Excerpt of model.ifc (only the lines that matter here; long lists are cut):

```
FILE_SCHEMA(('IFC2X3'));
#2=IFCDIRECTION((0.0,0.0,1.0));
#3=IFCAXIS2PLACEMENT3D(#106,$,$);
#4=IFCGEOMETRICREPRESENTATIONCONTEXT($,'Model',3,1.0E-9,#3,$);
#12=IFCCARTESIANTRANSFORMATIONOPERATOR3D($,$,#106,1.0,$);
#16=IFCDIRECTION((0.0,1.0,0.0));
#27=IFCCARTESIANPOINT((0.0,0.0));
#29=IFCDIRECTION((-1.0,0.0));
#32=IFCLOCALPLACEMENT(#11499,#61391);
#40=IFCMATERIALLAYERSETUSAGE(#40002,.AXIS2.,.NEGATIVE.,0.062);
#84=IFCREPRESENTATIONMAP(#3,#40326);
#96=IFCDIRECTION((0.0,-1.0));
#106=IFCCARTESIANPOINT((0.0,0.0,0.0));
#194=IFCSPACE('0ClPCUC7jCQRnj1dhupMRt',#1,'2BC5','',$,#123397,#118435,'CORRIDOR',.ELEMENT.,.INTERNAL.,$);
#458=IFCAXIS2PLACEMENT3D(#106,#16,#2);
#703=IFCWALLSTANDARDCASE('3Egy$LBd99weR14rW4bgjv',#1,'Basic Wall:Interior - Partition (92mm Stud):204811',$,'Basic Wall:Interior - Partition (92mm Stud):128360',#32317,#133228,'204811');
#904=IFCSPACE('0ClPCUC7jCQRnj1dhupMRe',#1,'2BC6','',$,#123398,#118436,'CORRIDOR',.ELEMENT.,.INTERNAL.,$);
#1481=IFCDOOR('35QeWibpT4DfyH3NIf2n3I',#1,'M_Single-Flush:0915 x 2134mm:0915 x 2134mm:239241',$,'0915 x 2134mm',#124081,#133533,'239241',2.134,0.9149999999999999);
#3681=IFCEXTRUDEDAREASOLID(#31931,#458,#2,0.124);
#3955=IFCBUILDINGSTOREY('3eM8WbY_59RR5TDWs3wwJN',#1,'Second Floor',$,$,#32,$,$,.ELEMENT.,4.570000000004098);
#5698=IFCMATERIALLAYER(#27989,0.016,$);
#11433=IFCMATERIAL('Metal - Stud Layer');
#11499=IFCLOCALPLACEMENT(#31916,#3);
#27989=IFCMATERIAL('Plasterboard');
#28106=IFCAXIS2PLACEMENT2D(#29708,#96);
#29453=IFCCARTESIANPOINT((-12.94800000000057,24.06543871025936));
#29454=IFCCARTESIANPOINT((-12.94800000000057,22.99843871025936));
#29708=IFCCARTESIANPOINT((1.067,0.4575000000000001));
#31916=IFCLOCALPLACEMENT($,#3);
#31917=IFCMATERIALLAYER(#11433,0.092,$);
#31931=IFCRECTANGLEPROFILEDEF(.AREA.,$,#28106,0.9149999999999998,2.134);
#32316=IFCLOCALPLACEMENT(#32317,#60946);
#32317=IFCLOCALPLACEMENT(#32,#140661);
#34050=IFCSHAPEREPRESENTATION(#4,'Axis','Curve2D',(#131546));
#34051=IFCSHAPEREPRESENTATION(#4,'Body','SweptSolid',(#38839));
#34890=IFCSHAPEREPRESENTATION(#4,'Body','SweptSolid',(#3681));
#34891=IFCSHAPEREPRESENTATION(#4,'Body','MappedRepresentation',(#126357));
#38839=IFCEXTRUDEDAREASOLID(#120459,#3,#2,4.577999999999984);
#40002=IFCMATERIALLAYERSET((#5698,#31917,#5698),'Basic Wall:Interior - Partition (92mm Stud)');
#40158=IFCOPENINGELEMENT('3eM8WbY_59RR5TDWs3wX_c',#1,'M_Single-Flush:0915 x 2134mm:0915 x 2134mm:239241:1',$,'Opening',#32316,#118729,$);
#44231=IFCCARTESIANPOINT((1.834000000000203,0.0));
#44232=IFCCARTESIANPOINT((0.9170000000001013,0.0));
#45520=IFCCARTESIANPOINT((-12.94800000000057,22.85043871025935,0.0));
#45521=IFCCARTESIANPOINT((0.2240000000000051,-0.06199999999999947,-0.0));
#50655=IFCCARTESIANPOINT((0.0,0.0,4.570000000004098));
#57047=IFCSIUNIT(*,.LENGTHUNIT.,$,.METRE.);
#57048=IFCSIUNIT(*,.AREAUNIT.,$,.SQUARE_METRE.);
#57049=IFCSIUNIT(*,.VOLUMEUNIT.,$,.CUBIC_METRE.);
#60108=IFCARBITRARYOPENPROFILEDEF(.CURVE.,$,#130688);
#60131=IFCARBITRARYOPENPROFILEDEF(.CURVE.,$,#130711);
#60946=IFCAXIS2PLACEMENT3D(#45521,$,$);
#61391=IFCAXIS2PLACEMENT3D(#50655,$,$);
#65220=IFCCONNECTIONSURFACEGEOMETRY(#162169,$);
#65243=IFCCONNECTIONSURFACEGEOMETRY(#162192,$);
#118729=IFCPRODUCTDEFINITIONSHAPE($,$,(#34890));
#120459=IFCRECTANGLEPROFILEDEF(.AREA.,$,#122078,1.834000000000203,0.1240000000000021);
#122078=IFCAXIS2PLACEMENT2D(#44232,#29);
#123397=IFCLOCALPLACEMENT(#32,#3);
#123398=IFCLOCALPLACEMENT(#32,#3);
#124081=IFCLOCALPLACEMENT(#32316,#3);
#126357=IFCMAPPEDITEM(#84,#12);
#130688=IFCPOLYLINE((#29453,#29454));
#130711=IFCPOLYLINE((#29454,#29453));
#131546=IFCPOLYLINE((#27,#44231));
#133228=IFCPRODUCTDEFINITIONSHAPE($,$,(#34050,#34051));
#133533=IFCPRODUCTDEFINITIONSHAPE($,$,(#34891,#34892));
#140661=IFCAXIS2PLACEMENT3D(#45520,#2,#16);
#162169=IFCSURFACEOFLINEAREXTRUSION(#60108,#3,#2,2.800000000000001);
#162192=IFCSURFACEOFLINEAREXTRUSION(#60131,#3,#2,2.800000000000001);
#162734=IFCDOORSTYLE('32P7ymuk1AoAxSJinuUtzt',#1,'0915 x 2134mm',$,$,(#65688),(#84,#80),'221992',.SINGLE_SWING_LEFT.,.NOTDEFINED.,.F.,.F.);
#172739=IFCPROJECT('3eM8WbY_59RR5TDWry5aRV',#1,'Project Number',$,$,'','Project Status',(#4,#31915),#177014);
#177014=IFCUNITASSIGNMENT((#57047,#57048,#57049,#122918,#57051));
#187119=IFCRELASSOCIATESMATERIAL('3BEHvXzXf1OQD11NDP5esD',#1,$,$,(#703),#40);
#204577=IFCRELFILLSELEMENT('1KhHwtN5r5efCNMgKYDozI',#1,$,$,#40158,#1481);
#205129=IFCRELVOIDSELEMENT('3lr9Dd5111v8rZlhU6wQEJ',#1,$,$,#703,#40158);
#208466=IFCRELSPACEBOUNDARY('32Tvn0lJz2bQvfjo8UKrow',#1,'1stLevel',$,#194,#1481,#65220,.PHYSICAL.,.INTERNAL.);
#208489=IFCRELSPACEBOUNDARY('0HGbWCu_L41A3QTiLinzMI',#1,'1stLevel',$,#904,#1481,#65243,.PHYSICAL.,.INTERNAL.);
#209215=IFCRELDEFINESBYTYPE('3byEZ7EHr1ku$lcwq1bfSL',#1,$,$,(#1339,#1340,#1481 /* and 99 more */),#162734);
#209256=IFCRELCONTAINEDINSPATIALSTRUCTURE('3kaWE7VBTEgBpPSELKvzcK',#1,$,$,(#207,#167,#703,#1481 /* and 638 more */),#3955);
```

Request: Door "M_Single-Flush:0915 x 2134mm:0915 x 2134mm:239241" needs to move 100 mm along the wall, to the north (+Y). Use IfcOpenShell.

```python
import numpy as np
import ifcopenshell
import ifcopenshell.api.geometry
import ifcopenshell.util.placement
import ifcopenshell.util.unit

model = ifcopenshell.open("model.ifc")
unit_scale = ifcopenshell.util.unit.calculate_unit_scale(model)

door = model.by_id(1481)
opening = door.FillsVoids[0].RelatingOpeningElement
wall = opening.VoidsElements[0].RelatingBuildingElement

wall_matrix = ifcopenshell.util.placement.get_local_placement(wall.ObjectPlacement)
shift = wall_matrix[:3, 0] * 0.1 / unit_scale
before = ifcopenshell.util.placement.get_local_placement(door.ObjectPlacement)[:3, 3].copy()

# The door is placed relative to its opening, so it follows when the opening moves.
matrix = ifcopenshell.util.placement.get_local_placement(opening.ObjectPlacement)
matrix[:3, 3] += shift
ifcopenshell.api.geometry.edit_object_placement(
    model, product=opening, matrix=matrix, is_si=False, should_transform_children=True
)

# Space boundary surfaces are stored in each space's coordinates; move them too.
for rel in door.ProvidesBoundaries:
    if not rel.ConnectionGeometry:
        continue
    surface = rel.ConnectionGeometry.SurfaceOnRelatingElement
    space_matrix = ifcopenshell.util.placement.get_local_placement(rel.RelatingSpace.ObjectPlacement)
    point = np.array(surface.Position.Location.Coordinates) + space_matrix[:3, :3].T @ shift
    surface.Position = model.createIfcAxis2Placement3D(
        model.createIfcCartesianPoint(point.tolist()), surface.Position.Axis, surface.Position.RefDirection
    )

after = ifcopenshell.util.placement.get_local_placement(door.ObjectPlacement)[:3, 3]
print("door moved by", (after - before).round(3) + 0.0)

model.write("model_rev.ifc")
```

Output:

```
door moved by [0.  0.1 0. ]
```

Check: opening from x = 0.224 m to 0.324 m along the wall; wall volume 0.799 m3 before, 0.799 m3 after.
